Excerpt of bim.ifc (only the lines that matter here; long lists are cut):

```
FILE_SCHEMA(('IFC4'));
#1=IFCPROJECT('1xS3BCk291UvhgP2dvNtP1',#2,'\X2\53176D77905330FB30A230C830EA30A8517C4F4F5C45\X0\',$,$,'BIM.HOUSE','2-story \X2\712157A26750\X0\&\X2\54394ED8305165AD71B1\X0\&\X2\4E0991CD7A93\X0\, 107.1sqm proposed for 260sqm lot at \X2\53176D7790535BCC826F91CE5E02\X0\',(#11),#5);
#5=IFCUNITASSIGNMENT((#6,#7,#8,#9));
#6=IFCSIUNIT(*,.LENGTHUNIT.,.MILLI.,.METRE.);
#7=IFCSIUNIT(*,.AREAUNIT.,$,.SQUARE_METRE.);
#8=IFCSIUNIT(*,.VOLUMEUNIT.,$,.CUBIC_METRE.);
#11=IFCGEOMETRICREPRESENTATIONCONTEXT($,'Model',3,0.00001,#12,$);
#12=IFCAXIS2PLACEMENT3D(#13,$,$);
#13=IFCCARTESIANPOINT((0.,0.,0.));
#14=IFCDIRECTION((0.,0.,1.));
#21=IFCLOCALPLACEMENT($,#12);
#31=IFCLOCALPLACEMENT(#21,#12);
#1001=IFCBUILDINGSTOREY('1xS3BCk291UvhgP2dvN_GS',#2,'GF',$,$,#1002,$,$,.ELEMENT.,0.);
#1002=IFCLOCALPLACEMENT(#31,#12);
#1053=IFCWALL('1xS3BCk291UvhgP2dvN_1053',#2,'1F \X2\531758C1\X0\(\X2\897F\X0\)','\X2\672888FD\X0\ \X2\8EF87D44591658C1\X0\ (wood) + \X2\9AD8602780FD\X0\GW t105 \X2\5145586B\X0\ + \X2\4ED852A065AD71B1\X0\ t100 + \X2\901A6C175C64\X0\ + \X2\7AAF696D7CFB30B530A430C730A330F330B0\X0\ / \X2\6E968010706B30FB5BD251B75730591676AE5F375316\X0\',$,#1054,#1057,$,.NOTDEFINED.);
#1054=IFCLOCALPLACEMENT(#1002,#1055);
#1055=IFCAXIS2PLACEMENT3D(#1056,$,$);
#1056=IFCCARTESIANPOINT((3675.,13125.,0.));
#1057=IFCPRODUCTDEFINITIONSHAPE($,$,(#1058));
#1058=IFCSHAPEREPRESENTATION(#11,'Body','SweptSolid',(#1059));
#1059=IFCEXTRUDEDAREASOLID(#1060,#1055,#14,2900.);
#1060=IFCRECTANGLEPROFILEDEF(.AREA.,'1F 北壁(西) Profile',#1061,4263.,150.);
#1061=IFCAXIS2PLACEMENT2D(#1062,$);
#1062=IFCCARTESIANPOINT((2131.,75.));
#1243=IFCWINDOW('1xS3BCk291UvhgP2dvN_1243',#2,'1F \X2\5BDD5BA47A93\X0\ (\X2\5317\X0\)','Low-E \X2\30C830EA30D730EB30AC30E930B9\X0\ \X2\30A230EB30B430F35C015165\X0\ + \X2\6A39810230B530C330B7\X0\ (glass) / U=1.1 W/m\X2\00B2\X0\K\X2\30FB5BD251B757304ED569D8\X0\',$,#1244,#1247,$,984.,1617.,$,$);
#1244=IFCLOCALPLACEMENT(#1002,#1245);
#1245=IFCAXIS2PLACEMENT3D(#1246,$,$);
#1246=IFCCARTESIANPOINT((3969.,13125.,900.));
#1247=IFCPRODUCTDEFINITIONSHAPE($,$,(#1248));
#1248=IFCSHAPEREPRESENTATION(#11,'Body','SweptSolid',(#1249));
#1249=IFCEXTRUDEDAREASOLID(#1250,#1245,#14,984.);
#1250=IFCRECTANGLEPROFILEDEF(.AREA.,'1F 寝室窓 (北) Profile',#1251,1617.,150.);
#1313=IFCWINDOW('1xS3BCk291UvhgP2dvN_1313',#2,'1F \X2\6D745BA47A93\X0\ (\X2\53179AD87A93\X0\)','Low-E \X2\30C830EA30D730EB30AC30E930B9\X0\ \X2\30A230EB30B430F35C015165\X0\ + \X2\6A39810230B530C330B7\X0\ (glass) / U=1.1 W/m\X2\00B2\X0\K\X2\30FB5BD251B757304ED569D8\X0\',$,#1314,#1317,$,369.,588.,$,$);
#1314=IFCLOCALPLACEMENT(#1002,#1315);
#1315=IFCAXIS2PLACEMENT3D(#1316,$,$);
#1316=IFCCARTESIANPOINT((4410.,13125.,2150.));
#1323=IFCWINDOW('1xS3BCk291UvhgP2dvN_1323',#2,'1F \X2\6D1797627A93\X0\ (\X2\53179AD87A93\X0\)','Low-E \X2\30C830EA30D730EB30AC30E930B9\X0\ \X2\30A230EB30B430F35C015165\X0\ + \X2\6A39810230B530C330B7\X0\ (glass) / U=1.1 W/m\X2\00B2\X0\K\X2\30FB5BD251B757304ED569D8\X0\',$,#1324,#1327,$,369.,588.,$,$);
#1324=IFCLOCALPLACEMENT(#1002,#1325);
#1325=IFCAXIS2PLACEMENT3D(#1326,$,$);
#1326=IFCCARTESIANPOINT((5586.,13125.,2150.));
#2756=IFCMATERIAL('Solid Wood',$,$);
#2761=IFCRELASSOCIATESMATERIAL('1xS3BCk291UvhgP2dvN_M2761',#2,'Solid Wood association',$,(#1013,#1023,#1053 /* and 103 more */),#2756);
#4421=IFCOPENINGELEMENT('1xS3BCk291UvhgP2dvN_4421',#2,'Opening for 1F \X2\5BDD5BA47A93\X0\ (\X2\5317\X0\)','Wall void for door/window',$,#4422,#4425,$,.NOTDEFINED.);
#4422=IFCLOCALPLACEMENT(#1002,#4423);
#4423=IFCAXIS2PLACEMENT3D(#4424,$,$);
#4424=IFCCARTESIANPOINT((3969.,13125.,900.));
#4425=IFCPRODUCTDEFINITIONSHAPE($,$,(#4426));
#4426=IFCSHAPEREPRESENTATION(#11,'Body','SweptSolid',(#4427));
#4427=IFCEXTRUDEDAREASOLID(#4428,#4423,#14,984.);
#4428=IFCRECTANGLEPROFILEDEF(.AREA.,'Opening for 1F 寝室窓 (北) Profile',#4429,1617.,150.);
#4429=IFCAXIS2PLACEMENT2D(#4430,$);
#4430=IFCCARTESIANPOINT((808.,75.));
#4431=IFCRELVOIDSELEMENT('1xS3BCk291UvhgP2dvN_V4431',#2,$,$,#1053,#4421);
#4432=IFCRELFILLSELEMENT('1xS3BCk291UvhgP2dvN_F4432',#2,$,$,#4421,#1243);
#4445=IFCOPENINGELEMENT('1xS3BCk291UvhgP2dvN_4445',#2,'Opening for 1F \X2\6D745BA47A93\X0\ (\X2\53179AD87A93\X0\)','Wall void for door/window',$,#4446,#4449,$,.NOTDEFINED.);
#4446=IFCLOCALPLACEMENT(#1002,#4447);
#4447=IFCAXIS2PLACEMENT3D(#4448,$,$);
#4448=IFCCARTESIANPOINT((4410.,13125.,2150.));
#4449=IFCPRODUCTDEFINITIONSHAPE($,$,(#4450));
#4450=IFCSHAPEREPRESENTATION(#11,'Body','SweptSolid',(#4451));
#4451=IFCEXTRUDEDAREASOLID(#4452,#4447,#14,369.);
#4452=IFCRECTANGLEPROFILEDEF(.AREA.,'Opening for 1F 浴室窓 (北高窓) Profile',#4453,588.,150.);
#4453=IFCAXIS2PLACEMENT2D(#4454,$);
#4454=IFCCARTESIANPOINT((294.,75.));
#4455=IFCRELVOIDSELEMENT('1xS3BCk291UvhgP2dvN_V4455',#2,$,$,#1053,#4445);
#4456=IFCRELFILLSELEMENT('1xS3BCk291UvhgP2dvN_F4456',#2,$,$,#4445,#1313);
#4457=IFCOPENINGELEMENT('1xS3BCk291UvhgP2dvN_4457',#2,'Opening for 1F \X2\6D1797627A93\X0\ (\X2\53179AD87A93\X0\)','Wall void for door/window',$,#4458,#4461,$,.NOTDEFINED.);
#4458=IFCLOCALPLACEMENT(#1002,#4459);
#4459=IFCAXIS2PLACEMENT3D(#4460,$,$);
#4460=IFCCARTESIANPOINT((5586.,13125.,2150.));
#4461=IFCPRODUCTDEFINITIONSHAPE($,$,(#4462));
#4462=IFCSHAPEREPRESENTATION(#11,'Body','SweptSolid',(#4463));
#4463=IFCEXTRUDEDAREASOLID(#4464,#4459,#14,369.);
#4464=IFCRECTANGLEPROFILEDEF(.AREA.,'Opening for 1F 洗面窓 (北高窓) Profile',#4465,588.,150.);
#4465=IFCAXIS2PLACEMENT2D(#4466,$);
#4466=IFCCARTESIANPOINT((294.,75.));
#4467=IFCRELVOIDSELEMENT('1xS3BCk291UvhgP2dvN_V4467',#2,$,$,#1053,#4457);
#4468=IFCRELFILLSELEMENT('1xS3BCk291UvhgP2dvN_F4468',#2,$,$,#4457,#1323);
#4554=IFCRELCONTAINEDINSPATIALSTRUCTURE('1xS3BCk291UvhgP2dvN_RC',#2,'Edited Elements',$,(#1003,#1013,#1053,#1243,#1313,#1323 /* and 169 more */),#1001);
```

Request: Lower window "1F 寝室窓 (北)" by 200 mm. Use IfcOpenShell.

```python
import numpy as np
import ifcopenshell
import ifcopenshell.api.geometry
import ifcopenshell.util.placement
import ifcopenshell.util.unit

model = ifcopenshell.open("bim.ifc")
unit_scale = ifcopenshell.util.unit.calculate_unit_scale(model)

window = model.by_guid("1xS3BCk291UvhgP2dvN_1243")
opening = window.FillsVoids[0].RelatingOpeningElement
dz = -0.2 / unit_scale

shift = np.array([0.0, 0.0, dz])
# The window is not placed relative to its opening, so move both.
for product in (opening, window):
    matrix = ifcopenshell.util.placement.get_local_placement(product.ObjectPlacement)
    matrix[:3, 3] += shift
    ifcopenshell.api.geometry.edit_object_placement(model, product=product, matrix=matrix, is_si=False)

print(f"moved by {dz * unit_scale:+.3f} m")

model.write("bim_edited.ifc")
```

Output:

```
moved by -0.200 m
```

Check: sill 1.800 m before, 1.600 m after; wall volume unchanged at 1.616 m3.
